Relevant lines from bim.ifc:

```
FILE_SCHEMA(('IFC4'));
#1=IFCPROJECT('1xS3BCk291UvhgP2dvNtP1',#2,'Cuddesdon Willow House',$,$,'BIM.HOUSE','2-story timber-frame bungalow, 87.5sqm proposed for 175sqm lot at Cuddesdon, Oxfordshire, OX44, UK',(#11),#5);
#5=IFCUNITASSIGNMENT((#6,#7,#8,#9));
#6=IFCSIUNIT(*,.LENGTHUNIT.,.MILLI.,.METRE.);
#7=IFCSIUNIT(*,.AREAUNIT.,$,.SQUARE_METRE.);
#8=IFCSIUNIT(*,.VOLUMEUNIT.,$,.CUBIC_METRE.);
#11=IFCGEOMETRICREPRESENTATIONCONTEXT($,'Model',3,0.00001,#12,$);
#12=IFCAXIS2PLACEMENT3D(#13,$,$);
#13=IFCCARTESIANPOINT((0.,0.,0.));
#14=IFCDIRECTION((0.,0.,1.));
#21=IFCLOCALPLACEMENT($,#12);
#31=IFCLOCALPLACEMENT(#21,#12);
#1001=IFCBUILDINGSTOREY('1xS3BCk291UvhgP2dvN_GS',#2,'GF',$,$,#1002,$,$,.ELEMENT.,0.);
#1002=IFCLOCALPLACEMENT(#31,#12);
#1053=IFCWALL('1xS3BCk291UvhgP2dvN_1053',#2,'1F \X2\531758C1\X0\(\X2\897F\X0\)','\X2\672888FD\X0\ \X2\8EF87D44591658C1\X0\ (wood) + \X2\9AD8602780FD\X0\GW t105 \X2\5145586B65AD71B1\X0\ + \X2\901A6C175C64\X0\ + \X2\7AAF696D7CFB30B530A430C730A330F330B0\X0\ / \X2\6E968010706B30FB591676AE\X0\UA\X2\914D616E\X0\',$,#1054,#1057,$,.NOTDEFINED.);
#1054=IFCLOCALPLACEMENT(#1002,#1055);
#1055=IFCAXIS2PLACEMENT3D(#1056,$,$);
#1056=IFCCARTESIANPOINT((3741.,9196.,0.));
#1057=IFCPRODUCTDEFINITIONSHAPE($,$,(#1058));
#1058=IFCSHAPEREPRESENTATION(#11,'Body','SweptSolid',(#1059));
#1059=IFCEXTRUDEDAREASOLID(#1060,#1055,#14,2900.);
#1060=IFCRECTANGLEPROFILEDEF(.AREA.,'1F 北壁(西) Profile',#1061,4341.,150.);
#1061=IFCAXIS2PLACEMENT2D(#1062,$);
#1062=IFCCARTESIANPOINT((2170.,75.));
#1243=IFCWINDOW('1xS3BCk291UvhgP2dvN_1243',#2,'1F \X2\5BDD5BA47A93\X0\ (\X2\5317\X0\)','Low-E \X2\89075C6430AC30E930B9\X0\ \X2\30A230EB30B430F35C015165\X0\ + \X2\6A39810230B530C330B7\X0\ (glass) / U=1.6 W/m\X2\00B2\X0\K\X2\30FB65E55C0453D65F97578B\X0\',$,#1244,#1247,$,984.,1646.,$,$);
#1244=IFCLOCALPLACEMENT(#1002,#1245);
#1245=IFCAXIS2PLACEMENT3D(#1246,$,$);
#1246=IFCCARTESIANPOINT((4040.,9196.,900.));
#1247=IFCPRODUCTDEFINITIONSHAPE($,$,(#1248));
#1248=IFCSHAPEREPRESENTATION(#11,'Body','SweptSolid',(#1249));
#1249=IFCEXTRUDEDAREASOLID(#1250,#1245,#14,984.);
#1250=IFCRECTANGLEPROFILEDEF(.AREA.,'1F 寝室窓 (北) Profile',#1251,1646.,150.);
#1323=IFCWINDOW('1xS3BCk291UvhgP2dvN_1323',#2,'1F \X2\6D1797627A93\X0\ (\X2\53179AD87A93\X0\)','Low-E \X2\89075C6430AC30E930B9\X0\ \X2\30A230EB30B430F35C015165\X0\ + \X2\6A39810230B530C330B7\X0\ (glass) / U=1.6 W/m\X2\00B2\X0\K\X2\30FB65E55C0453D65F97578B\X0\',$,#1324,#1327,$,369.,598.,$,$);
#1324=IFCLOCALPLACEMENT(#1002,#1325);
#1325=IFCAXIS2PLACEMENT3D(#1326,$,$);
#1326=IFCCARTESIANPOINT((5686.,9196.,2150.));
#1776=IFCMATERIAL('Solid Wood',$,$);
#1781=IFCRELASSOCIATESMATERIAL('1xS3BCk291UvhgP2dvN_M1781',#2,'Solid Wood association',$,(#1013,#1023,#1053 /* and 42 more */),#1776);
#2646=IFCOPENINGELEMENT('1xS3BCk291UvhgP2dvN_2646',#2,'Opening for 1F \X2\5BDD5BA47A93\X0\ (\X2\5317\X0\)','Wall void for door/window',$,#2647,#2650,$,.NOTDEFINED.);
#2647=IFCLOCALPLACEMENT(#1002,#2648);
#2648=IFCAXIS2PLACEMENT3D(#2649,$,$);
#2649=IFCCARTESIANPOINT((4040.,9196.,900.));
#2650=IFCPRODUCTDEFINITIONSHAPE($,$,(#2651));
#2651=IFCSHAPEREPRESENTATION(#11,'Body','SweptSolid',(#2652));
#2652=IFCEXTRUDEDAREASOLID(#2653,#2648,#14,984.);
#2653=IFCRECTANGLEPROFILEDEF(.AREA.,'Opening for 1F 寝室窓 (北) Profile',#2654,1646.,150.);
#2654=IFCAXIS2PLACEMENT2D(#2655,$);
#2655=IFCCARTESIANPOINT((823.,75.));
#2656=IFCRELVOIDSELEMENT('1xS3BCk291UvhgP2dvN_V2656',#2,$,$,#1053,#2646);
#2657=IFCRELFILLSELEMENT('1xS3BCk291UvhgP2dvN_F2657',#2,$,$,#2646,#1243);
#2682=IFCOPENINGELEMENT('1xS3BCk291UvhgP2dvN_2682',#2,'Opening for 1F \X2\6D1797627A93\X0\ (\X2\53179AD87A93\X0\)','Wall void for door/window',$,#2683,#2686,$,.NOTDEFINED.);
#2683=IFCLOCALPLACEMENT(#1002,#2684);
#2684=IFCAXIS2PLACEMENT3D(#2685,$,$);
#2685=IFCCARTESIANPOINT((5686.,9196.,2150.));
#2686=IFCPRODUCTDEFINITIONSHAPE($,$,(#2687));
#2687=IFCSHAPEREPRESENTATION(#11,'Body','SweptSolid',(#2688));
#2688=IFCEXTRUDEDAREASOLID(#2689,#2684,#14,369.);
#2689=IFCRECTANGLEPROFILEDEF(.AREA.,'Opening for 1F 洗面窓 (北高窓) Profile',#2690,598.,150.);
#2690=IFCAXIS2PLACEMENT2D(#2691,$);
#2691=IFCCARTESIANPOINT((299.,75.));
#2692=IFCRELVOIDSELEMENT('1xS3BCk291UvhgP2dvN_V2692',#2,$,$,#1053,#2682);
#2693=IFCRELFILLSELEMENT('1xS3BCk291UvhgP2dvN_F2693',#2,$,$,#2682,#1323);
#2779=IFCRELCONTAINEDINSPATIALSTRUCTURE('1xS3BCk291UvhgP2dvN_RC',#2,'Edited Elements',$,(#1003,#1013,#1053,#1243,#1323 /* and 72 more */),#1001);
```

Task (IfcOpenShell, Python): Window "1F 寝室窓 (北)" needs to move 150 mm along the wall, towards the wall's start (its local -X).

```python
import ifcopenshell
import ifcopenshell.api.geometry
import ifcopenshell.util.placement

model = ifcopenshell.open("bim.ifc")

window = model.by_id(1243)
opening = window.FillsVoids[0].RelatingOpeningElement
wall = opening.VoidsElements[0].RelatingBuildingElement

wall_matrix = ifcopenshell.util.placement.get_local_placement(wall.ObjectPlacement)
shift = wall_matrix[:3, 0] * -150.0
before = ifcopenshell.util.placement.get_local_placement(window.ObjectPlacement)[:3, 3].copy()

# The window is not placed relative to its opening, so move both.
for product in (opening, window):
    matrix = ifcopenshell.util.placement.get_local_placement(product.ObjectPlacement)
    matrix[:3, 3] += shift
    ifcopenshell.api.geometry.edit_object_placement(model, product=product, matrix=matrix, is_si=False)

after = ifcopenshell.util.placement.get_local_placement(window.ObjectPlacement)[:3, 3]
print("window moved by", (after - before).round(3) + 0.0)

model.write("bim_updated.ifc")
```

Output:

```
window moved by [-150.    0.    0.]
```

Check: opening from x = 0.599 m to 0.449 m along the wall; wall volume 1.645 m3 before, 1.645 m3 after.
